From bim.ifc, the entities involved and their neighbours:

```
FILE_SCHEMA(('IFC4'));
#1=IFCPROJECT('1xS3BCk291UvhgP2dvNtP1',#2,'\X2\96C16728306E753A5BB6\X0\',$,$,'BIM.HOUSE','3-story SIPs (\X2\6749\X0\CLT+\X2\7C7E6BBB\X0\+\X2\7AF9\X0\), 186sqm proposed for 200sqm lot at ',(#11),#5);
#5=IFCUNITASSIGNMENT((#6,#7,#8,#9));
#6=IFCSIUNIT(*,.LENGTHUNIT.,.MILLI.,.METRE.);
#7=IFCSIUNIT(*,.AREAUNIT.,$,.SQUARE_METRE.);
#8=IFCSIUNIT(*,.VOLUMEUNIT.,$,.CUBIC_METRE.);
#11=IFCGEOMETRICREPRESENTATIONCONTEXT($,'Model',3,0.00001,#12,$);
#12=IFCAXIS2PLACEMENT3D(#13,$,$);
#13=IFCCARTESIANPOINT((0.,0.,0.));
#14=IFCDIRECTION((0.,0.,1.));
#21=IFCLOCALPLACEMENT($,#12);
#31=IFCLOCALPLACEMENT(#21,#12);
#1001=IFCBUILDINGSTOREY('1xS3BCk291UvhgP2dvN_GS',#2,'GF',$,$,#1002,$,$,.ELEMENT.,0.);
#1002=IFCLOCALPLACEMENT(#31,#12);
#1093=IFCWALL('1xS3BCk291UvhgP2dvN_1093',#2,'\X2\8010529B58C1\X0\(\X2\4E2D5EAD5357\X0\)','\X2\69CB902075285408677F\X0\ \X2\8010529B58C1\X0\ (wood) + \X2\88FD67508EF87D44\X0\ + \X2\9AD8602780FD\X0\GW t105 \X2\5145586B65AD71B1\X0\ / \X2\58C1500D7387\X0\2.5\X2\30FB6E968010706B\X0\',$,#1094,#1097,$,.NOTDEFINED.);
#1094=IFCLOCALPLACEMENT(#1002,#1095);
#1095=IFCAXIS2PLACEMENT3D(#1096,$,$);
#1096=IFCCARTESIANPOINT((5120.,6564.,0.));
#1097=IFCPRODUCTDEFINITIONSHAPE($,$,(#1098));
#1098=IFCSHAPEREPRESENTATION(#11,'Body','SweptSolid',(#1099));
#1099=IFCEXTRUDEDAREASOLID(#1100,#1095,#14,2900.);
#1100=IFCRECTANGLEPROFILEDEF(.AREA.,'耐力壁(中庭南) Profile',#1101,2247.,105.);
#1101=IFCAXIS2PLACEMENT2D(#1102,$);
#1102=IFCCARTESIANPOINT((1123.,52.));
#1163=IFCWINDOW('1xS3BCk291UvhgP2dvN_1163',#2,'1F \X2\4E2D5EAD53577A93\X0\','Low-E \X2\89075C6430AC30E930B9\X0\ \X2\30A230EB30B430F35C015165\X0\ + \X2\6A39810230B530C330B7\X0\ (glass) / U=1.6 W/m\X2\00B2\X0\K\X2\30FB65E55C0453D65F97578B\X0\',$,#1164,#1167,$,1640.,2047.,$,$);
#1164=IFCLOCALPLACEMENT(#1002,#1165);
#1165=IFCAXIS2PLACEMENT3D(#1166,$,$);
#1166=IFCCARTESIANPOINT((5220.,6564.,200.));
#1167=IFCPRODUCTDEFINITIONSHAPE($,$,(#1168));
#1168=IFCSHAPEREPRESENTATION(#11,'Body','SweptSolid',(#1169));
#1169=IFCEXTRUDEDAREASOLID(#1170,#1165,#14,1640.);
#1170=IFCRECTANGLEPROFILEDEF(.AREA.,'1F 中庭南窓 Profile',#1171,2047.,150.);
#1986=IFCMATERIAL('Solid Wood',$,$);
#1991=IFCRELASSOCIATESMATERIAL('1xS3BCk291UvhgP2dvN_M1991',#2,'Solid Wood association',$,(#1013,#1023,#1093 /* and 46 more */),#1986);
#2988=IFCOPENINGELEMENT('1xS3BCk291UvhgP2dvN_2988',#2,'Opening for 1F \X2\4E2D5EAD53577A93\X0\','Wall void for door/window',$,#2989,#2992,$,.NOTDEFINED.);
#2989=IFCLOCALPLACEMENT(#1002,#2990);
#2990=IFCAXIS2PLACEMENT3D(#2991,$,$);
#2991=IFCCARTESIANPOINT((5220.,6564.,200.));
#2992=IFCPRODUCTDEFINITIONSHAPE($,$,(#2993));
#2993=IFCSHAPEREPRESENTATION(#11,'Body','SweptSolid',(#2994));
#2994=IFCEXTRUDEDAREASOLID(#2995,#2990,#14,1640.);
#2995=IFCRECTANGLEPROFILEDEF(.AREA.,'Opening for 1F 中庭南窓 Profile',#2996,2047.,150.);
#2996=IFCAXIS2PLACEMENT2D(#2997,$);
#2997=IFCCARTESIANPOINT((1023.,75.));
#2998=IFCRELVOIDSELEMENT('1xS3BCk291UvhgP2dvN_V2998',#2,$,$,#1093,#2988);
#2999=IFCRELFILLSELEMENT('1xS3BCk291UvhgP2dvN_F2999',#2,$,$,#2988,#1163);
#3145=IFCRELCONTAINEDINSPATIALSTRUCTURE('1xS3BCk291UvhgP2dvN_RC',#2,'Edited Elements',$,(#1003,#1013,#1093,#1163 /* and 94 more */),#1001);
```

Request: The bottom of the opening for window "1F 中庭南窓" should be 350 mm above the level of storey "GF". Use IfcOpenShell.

```python
import numpy as np
import ifcopenshell
import ifcopenshell.api.geometry
import ifcopenshell.geom
import ifcopenshell.util.element
import ifcopenshell.util.placement
import ifcopenshell.util.shape
import ifcopenshell.util.unit

model = ifcopenshell.open("bim.ifc")
unit_scale = ifcopenshell.util.unit.calculate_unit_scale(model)

window = model.by_guid("1xS3BCk291UvhgP2dvN_1163")
opening = window.FillsVoids[0].RelatingOpeningElement
storey = ifcopenshell.util.element.get_container(window, ifc_class="IfcBuildingStorey")
level = ifcopenshell.util.placement.get_local_placement(storey.ObjectPlacement)[2, 3]

# The opening's origin need not be at the sill, so measure its lowest point.
shape = ifcopenshell.geom.create_shape(ifcopenshell.geom.settings(), opening)
bottom = ifcopenshell.util.shape.get_shape_bottom_elevation(shape, shape.geometry) / unit_scale
dz = level + 350.0 - bottom

shift = np.array([0.0, 0.0, dz])
# The window is not placed relative to its opening, so move both.
for product in (opening, window):
    matrix = ifcopenshell.util.placement.get_local_placement(product.ObjectPlacement)
    matrix[:3, 3] += shift
    ifcopenshell.api.geometry.edit_object_placement(model, product=product, matrix=matrix, is_si=False)

print(f"moved by {dz * unit_scale:+.3f} m")

model.write("bim_rev.ifc")
```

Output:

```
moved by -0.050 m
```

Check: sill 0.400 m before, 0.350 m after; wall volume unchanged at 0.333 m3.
